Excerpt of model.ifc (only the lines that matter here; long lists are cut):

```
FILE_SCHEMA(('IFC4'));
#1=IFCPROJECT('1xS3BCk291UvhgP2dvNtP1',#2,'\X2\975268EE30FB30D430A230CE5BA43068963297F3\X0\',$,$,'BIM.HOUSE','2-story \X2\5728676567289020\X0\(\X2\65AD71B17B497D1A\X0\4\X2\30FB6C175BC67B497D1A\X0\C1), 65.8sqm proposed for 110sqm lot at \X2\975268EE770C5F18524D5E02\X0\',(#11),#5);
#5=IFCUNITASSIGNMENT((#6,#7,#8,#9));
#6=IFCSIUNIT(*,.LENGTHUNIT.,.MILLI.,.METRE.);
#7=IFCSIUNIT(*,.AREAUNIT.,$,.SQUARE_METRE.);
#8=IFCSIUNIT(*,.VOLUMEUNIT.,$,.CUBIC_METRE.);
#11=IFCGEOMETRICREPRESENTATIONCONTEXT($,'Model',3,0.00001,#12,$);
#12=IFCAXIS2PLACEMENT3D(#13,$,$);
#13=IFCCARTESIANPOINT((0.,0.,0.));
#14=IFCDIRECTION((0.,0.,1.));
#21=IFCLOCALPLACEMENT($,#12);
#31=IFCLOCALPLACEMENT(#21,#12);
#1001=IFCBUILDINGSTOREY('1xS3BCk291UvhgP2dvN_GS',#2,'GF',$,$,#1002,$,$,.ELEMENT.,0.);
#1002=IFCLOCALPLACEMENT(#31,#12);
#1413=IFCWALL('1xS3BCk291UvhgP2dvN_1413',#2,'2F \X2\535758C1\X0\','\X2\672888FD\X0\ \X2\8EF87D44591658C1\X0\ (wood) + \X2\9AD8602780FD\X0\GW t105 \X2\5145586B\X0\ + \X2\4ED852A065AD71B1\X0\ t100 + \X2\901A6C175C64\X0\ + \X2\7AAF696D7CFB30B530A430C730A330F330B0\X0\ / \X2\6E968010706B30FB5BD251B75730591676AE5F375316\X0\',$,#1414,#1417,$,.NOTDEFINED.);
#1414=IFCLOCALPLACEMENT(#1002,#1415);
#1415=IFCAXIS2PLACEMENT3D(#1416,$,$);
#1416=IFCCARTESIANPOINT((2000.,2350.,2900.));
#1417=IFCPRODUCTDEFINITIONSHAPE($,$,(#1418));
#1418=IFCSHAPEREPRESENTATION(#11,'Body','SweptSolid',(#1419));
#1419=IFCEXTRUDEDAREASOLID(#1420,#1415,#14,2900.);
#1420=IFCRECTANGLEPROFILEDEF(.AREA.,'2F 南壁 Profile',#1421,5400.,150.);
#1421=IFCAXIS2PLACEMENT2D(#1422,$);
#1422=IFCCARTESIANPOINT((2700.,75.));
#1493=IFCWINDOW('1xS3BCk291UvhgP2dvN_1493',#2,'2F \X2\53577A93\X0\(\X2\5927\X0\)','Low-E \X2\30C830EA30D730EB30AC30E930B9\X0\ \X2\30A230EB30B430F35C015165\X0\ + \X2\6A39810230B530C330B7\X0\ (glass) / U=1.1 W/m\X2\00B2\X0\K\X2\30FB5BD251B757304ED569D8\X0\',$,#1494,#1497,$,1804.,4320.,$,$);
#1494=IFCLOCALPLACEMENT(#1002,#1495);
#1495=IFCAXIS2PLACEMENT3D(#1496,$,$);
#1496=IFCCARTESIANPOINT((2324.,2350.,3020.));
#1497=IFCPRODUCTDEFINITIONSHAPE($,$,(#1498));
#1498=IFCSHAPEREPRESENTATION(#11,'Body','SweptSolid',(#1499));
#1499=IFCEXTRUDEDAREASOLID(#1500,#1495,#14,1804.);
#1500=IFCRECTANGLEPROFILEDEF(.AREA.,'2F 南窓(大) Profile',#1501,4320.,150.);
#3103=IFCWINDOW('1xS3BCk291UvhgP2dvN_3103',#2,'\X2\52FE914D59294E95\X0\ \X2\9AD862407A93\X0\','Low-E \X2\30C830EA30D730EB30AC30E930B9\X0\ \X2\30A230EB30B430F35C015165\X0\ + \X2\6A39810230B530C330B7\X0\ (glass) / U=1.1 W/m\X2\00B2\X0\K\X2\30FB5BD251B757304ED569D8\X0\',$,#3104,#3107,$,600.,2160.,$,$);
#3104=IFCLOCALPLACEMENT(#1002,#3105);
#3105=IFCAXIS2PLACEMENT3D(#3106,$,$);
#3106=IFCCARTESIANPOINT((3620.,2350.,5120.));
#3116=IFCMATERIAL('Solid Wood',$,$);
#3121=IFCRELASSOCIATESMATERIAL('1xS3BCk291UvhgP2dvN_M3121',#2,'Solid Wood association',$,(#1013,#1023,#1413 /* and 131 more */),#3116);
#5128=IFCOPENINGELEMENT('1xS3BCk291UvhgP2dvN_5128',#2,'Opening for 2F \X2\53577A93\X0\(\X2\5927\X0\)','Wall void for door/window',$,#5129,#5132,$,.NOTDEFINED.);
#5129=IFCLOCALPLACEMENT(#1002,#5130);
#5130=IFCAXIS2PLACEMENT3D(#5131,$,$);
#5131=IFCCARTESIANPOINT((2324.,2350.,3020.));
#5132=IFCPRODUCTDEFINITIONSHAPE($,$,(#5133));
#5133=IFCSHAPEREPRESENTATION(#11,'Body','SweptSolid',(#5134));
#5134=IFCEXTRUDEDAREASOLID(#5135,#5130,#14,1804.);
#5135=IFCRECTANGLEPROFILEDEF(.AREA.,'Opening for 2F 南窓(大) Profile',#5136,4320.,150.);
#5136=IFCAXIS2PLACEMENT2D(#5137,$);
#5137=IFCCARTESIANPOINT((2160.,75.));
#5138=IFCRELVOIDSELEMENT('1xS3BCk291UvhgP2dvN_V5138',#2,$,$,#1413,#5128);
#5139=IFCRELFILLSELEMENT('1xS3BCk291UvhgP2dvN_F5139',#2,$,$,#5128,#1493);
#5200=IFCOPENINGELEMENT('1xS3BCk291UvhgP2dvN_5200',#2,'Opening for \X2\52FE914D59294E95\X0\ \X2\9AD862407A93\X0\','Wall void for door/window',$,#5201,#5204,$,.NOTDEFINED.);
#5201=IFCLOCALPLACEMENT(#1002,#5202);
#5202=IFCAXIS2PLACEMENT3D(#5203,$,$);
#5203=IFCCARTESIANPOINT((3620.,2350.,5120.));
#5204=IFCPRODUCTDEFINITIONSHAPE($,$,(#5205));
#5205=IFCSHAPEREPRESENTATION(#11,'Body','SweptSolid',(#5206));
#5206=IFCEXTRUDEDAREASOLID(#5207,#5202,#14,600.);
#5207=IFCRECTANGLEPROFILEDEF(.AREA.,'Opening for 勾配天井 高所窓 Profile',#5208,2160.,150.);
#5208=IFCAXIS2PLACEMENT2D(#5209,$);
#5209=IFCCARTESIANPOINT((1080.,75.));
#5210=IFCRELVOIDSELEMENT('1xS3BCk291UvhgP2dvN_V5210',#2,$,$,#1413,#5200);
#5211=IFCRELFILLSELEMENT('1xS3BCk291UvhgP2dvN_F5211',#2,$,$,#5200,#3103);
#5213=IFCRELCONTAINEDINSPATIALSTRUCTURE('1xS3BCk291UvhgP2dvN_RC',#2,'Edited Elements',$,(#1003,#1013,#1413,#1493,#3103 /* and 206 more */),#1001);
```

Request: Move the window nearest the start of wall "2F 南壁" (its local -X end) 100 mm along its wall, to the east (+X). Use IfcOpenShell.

```python
import ifcopenshell
import ifcopenshell.api.geometry
import ifcopenshell.util.placement

model = ifcopenshell.open("model.ifc")

window = model.by_id(1493)
opening = window.FillsVoids[0].RelatingOpeningElement
wall = opening.VoidsElements[0].RelatingBuildingElement

wall_matrix = ifcopenshell.util.placement.get_local_placement(wall.ObjectPlacement)
shift = wall_matrix[:3, 0] * 100.0
before = ifcopenshell.util.placement.get_local_placement(window.ObjectPlacement)[:3, 3].copy()

# The window is not placed relative to its opening, so move both.
for product in (opening, window):
    matrix = ifcopenshell.util.placement.get_local_placement(product.ObjectPlacement)
    matrix[:3, 3] += shift
    ifcopenshell.api.geometry.edit_object_placement(model, product=product, matrix=matrix, is_si=False)

after = ifcopenshell.util.placement.get_local_placement(window.ObjectPlacement)[:3, 3]
print("window moved by", (after - before).round(3) + 0.0)

model.write("model_v2.ifc")
```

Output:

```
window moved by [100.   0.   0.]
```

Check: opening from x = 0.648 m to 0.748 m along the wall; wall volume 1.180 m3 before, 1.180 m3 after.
